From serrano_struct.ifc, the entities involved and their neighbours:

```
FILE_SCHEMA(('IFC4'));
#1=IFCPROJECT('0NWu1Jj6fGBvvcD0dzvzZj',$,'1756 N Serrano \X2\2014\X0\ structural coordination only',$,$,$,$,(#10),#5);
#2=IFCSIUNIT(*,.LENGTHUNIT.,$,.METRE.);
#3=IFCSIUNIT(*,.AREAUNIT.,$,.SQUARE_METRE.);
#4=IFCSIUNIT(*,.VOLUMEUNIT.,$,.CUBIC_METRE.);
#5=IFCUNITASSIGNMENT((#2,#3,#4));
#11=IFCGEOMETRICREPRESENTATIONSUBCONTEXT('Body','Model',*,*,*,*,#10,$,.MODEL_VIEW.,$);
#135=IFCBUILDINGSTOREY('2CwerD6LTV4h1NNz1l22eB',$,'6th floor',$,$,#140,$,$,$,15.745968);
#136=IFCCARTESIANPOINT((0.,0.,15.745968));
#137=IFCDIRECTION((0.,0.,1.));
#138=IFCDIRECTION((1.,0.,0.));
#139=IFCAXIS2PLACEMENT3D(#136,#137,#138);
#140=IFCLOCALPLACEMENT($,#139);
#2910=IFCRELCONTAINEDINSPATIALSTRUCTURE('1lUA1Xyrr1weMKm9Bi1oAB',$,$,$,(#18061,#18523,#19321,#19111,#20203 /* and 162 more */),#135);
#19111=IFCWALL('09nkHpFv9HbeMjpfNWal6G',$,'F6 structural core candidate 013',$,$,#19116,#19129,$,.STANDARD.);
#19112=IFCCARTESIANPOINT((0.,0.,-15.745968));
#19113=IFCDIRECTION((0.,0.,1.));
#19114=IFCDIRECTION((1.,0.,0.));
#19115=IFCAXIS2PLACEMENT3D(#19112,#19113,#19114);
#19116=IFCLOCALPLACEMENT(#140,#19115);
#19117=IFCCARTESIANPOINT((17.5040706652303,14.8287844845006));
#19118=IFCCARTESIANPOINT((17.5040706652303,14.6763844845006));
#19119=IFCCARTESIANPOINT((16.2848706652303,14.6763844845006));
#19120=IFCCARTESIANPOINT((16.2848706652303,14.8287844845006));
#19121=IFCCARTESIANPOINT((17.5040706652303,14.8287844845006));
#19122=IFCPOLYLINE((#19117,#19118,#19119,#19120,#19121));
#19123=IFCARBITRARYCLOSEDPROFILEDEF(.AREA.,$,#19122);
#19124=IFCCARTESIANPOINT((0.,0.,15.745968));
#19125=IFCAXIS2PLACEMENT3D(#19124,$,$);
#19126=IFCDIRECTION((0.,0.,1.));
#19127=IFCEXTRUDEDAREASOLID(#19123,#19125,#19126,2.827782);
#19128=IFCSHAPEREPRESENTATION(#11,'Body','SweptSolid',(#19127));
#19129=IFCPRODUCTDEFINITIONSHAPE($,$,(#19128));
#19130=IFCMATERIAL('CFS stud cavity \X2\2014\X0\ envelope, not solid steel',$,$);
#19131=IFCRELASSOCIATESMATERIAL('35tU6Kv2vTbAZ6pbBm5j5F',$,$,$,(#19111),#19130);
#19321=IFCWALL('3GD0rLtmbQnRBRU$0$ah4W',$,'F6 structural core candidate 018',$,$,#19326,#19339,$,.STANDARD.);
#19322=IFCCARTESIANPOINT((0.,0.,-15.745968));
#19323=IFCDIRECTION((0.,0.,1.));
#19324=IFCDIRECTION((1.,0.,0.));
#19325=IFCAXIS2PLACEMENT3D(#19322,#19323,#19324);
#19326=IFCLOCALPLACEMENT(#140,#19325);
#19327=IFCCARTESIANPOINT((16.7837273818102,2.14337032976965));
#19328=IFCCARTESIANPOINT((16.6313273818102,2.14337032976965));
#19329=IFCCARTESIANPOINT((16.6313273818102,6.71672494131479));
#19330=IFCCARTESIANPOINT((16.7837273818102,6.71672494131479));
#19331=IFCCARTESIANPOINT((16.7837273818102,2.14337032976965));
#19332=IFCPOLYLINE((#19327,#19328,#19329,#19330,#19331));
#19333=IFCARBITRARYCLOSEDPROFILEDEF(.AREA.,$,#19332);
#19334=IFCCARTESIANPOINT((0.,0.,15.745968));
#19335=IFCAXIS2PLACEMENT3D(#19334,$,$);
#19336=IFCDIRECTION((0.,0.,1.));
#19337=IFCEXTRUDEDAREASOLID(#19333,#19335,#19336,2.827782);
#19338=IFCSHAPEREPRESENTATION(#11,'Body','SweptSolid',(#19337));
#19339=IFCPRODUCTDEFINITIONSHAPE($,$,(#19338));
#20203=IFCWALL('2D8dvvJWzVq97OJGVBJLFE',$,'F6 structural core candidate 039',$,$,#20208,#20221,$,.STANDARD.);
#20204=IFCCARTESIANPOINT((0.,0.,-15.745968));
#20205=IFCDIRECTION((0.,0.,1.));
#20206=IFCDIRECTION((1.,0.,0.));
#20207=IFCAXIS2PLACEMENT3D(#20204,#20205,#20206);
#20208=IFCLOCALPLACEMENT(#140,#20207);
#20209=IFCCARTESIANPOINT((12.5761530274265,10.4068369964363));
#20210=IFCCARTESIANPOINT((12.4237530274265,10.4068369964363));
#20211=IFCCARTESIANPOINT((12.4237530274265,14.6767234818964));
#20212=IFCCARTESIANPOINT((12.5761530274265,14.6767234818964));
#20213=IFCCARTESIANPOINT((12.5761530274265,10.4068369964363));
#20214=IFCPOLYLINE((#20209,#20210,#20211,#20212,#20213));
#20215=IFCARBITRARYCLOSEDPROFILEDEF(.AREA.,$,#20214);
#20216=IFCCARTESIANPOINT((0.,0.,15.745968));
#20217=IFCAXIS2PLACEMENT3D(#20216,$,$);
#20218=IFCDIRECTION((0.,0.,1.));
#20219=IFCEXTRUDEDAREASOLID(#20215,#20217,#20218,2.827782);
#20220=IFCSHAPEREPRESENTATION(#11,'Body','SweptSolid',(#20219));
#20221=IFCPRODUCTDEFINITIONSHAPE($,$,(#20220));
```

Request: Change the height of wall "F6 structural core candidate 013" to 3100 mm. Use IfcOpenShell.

```python
import ifcopenshell
import ifcopenshell.geom
import ifcopenshell.util.representation
import ifcopenshell.util.shape
import ifcopenshell.util.unit

model = ifcopenshell.open("serrano_struct.ifc")
unit_scale = ifcopenshell.util.unit.calculate_unit_scale(model)
settings = ifcopenshell.geom.settings()


def volume(element):
    """Net volume in cubic metres, openings subtracted."""
    shape = ifcopenshell.geom.create_shape(settings, element)
    return ifcopenshell.util.shape.get_volume(shape.geometry)


wall = model.by_id(19111)
before = volume(wall)

body = ifcopenshell.util.representation.get_representation(wall, "Model", "Body")
solid = body.Items[0]
old_height = solid.Depth
solid.Depth = 3.1 / unit_scale
after = volume(wall)

print(f"height {old_height:g} -> {solid.Depth:g}, volume {before:.3f} -> {after:.3f} m3")

model.write("serrano_struct_rev.ifc")
```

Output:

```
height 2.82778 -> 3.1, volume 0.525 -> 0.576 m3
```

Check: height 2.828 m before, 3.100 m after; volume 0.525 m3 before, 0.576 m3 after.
